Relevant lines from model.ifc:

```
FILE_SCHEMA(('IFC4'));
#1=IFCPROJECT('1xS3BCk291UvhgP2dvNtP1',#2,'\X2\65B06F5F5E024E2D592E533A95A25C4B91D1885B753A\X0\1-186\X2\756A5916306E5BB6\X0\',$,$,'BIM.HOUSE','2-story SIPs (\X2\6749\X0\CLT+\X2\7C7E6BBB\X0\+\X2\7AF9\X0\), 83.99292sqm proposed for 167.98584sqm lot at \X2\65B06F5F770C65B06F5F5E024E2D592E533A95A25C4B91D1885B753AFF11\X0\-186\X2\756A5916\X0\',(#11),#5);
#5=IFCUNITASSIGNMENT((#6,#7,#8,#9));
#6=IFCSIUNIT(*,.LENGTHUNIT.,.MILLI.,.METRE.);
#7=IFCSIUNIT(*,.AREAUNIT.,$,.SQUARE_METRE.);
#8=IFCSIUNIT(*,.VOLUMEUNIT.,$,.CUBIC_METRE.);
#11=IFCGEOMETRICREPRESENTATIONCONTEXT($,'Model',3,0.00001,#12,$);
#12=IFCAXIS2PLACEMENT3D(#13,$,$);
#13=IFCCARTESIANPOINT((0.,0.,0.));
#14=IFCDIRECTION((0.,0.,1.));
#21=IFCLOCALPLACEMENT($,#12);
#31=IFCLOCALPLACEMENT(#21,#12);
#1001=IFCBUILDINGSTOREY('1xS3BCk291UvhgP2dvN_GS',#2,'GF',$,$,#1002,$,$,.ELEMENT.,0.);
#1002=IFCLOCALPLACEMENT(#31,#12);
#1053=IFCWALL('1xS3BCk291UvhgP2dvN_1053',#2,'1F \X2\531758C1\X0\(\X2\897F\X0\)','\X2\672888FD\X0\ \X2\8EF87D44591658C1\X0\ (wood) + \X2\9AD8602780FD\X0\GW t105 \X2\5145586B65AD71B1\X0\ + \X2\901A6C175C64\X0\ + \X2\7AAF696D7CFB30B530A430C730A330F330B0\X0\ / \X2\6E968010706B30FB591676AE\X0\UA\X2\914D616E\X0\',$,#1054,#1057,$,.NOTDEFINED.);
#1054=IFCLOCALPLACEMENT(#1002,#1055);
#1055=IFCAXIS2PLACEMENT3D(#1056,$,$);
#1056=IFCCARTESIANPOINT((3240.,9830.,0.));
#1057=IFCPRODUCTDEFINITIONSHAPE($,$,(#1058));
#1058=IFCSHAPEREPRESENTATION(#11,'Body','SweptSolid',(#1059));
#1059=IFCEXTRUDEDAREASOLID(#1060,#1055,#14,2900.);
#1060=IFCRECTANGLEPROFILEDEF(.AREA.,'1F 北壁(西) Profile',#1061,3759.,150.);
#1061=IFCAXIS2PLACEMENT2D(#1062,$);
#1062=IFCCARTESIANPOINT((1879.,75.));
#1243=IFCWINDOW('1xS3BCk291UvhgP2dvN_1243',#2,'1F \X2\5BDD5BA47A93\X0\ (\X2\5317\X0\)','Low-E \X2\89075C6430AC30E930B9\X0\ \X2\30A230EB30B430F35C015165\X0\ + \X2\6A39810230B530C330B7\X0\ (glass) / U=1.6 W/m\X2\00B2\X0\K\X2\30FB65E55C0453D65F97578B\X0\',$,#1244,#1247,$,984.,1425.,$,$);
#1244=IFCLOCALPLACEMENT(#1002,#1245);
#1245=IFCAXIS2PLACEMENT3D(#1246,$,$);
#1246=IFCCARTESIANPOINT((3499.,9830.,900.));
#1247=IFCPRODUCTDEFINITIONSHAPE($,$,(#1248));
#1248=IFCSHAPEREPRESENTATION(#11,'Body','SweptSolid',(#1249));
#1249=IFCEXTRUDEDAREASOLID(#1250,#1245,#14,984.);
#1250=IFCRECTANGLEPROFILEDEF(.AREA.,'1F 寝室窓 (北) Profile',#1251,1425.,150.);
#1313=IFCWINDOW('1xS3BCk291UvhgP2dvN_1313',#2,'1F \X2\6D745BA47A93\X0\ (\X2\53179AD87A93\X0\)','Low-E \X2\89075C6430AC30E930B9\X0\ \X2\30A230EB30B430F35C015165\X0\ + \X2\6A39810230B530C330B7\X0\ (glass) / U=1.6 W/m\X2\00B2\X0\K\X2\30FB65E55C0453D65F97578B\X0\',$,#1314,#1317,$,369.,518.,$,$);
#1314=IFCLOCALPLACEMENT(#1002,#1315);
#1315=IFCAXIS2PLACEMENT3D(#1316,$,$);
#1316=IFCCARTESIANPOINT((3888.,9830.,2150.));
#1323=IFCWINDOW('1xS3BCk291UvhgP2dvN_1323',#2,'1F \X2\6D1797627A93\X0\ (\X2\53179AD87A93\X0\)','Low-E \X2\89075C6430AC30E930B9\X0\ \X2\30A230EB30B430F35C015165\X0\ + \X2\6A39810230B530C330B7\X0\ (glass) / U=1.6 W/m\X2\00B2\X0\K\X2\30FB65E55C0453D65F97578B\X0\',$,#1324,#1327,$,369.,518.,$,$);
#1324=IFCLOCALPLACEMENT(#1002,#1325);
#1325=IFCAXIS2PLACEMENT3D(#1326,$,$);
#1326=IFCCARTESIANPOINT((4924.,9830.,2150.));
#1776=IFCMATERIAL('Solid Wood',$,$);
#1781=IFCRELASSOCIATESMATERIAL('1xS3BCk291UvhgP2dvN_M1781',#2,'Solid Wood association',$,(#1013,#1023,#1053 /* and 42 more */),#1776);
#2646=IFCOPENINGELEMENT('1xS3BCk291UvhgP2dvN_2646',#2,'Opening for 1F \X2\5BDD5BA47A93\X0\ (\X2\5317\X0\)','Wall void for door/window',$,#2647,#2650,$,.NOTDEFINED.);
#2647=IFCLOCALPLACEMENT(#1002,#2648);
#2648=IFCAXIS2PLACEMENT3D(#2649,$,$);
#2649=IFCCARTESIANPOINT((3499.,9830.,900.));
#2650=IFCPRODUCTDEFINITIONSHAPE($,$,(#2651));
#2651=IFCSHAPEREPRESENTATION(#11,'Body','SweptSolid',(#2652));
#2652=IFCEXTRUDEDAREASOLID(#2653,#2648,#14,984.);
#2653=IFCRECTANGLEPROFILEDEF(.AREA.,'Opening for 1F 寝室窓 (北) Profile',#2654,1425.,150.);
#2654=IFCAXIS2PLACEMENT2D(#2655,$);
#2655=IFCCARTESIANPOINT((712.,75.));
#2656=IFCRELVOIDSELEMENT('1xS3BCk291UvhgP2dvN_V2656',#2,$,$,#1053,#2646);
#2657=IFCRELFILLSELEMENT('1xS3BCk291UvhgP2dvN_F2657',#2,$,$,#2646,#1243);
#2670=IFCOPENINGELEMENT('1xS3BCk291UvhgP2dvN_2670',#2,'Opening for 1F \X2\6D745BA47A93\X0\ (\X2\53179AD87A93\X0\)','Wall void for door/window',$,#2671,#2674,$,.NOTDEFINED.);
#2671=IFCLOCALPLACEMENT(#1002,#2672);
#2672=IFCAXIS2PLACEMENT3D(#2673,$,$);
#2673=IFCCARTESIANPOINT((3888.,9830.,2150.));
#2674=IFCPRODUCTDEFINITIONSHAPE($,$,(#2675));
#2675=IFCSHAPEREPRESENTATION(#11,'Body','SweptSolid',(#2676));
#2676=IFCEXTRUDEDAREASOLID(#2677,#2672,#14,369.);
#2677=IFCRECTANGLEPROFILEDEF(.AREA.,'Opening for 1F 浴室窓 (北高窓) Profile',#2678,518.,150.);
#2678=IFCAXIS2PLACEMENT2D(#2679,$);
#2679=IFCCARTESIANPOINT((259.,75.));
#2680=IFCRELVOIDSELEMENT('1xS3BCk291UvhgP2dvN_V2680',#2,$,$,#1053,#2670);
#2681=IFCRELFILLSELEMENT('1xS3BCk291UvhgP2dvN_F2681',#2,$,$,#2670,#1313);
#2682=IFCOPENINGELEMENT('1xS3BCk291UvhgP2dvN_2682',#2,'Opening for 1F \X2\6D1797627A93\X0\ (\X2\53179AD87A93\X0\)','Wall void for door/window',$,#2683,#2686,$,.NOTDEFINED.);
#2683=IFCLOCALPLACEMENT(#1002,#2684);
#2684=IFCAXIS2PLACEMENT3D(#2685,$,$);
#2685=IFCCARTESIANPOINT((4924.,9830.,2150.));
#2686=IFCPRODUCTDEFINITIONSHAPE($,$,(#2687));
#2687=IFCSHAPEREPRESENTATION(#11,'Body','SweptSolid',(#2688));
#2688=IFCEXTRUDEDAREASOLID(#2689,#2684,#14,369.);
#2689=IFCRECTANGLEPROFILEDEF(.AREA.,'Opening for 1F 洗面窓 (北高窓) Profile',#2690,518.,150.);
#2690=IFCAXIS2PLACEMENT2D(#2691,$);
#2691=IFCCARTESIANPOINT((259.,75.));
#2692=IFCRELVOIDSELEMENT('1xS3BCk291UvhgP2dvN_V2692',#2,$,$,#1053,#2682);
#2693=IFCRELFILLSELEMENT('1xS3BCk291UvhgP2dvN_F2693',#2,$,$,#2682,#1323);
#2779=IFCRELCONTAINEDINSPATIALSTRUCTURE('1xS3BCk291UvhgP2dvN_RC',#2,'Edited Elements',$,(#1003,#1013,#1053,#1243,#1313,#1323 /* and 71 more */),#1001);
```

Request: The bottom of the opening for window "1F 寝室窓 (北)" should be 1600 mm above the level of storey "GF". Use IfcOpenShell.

```python
import numpy as np
import ifcopenshell
import ifcopenshell.api.geometry
import ifcopenshell.geom
import ifcopenshell.util.element
import ifcopenshell.util.placement
import ifcopenshell.util.shape
import ifcopenshell.util.unit

model = ifcopenshell.open("model.ifc")
unit_scale = ifcopenshell.util.unit.calculate_unit_scale(model)

window = model.by_id(1243)
opening = window.FillsVoids[0].RelatingOpeningElement
storey = ifcopenshell.util.element.get_container(window, ifc_class="IfcBuildingStorey")
level = ifcopenshell.util.placement.get_local_placement(storey.ObjectPlacement)[2, 3]

# The opening's origin need not be at the sill, so measure its lowest point.
shape = ifcopenshell.geom.create_shape(ifcopenshell.geom.settings(), opening)
bottom = ifcopenshell.util.shape.get_shape_bottom_elevation(shape, shape.geometry) / unit_scale
dz = level + 1.6 / unit_scale - bottom

shift = np.array([0.0, 0.0, dz])
# The window is not placed relative to its opening, so move both.
for product in (opening, window):
    matrix = ifcopenshell.util.placement.get_local_placement(product.ObjectPlacement)
    matrix[:3, 3] += shift
    ifcopenshell.api.geometry.edit_object_placement(model, product=product, matrix=matrix, is_si=False)

print(f"moved by {dz * unit_scale:+.3f} m")

model.write("model_v2.ifc")
```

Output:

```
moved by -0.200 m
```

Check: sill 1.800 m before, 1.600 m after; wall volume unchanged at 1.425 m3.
